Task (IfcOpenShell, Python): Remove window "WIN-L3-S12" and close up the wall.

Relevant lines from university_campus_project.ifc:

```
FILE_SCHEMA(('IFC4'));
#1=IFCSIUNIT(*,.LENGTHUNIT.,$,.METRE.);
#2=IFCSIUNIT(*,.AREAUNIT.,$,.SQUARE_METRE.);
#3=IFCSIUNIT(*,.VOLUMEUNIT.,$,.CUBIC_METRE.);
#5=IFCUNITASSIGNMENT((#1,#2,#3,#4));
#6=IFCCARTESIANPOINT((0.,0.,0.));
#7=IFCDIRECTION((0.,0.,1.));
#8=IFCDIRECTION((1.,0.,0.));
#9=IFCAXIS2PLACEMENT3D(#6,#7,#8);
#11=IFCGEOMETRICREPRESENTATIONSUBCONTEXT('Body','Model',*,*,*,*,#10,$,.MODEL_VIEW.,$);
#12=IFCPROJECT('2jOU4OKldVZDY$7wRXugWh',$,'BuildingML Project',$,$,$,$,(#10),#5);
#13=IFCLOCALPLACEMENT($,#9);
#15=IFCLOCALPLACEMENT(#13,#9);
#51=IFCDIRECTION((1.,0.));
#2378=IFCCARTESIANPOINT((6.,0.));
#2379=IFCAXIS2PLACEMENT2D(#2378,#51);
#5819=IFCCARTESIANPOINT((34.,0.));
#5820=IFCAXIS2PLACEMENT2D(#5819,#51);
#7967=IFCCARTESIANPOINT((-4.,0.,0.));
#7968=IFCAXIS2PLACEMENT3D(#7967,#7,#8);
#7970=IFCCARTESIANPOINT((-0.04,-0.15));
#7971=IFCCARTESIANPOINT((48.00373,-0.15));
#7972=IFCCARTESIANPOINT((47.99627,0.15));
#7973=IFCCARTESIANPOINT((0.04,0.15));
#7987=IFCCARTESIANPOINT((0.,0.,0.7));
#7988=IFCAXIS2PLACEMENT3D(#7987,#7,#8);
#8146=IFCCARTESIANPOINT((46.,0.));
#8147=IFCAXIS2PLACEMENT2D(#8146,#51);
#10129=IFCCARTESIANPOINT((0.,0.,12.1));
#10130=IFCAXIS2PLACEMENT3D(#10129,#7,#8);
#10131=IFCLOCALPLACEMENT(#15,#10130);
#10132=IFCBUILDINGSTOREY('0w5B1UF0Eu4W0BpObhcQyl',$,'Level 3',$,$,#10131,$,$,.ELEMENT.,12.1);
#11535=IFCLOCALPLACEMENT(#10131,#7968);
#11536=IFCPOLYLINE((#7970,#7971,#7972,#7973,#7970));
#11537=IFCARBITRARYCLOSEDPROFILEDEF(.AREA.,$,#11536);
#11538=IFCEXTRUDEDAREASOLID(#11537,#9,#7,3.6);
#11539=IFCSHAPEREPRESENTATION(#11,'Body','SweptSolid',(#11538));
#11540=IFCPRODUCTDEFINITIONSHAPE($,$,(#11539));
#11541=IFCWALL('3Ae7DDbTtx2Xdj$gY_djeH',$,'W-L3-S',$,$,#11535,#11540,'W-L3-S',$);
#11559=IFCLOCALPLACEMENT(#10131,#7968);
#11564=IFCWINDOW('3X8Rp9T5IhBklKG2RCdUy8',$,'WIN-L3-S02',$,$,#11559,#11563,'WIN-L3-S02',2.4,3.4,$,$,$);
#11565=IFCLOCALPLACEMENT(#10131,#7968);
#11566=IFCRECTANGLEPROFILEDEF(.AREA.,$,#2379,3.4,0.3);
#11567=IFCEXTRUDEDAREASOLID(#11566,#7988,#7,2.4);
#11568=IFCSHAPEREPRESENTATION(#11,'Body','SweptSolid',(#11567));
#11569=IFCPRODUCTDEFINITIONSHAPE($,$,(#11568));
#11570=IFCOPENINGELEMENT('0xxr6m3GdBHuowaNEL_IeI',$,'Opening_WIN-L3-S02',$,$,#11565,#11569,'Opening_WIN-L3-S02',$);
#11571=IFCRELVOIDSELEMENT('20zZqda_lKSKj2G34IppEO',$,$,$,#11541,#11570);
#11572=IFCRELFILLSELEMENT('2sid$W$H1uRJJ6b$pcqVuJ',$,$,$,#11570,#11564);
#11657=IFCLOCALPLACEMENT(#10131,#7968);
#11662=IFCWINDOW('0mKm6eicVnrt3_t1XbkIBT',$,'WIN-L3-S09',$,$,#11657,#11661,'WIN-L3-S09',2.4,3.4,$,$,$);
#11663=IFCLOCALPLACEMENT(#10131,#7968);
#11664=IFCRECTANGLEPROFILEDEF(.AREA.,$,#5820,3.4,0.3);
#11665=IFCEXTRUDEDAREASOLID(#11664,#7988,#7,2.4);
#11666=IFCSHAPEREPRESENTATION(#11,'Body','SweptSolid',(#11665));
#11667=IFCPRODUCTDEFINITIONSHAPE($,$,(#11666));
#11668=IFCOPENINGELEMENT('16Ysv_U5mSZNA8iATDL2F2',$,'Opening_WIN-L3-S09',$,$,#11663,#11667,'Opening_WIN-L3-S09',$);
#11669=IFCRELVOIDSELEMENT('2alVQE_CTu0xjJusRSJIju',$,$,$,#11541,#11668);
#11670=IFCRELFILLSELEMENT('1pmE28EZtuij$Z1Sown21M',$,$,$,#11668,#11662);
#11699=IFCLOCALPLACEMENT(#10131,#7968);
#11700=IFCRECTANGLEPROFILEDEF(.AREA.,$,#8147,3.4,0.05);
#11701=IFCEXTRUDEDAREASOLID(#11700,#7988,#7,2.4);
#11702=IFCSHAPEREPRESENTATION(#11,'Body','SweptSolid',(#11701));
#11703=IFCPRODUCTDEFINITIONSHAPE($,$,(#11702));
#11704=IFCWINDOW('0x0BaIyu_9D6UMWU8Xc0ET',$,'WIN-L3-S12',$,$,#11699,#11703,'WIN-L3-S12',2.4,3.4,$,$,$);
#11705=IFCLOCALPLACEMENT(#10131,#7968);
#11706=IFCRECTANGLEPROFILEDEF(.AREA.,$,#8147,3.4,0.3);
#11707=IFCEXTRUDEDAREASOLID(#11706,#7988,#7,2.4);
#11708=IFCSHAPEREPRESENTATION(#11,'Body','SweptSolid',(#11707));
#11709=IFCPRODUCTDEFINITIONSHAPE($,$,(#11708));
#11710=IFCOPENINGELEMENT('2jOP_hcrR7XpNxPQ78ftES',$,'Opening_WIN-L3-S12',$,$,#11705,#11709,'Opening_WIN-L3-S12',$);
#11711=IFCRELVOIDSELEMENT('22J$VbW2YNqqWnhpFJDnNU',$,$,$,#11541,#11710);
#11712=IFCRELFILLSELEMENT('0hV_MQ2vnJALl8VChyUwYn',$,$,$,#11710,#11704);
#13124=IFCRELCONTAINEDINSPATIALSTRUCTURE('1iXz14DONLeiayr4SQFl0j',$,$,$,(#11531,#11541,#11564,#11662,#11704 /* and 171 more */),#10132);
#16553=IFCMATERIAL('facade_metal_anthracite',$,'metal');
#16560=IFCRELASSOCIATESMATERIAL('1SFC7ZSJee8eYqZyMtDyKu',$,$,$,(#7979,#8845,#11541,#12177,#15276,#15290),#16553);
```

```python
import ifcopenshell
import ifcopenshell.api.feature
import ifcopenshell.api.root
import ifcopenshell.geom
import ifcopenshell.util.shape

model = ifcopenshell.open("university_campus_project.ifc")
settings = ifcopenshell.geom.settings()


def volume(element):
    """Net volume in cubic metres, openings subtracted."""
    shape = ifcopenshell.geom.create_shape(settings, element)
    return ifcopenshell.util.shape.get_volume(shape.geometry)


window = model.by_guid("0x0BaIyu_9D6UMWU8Xc0ET")
opening = window.FillsVoids[0].RelatingOpeningElement
wall = opening.VoidsElements[0].RelatingBuildingElement
before = volume(wall)

ifcopenshell.api.root.remove_product(model, product=window)
ifcopenshell.api.feature.remove_feature(model, feature=opening)

after = volume(wall)

print(f"wall volume {before:.3f} -> {after:.3f} m3")

model.write("university_campus_project_updated.ifc")
```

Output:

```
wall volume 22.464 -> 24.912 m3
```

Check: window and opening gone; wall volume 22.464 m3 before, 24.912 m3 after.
